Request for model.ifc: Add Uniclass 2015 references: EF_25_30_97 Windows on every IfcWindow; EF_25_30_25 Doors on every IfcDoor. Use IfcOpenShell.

First a look at what the model holds.

```python
import ifcopenshell

model = ifcopenshell.open("model.ifc")
print(model.schema)
print("classifications:", [c.Name for c in model.by_type("IfcClassification")])
for ifc_class in ("IfcDoor", "IfcRoof", "IfcStair", "IfcWall", "IfcWindow"):
    print(ifc_class, len(model.by_type(ifc_class)))
```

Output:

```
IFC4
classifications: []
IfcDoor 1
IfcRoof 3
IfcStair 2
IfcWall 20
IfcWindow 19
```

```python
import ifcopenshell
import ifcopenshell.api.classification

model = ifcopenshell.open("model.ifc")

system = ifcopenshell.api.classification.add_classification(model, classification="Uniclass 2015")

codes = {
    "IfcWindow": ("EF_25_30_97", "Windows"),
    "IfcDoor": ("EF_25_30_25", "Doors"),
}
for ifc_class, (code, name) in codes.items():
    products = model.by_type(ifc_class)
    ifcopenshell.api.classification.add_reference(
        model, products=products, classification=system, identification=code, name=name
    )
    print(code, len(products))

model.write("model_edited.ifc")
```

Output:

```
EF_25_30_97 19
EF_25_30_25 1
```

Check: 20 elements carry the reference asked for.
